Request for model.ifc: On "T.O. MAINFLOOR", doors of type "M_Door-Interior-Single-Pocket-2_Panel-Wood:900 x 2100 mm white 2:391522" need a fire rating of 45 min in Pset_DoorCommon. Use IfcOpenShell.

First a look at what the model holds.

```python
import ifcopenshell
import ifcopenshell.util.element

model = ifcopenshell.open("model.ifc")
print(model.schema)
storey = next(s for s in model.by_type("IfcBuildingStorey") if s.Name == "T.O. MAINFLOOR")
doors = [e for e in ifcopenshell.util.element.get_decomposition(storey) if e.is_a("IfcDoor")]
seen = {}
for e in doors:
    element_type = ifcopenshell.util.element.get_type(e)
    key = (element_type.Name if element_type != e and element_type else None, ifcopenshell.util.element.get_pset(e, "Pset_DoorCommon", "FireRating"))
    seen[key] = seen.get(key, 0) + 1
for (name, value), count in sorted(seen.items(), key=str):
    print(count, "x", name, "|", value)
```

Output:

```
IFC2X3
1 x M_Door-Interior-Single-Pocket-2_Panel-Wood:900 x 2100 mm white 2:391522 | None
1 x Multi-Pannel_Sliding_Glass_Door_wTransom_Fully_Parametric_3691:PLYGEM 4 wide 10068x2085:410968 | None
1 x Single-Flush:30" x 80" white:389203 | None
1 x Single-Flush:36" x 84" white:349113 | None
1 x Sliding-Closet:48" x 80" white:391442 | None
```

```python
import ifcopenshell
import ifcopenshell.api.pset
import ifcopenshell.util.element

model = ifcopenshell.open("model.ifc")

storey = next(s for s in model.by_type("IfcBuildingStorey") if s.Name == "T.O. MAINFLOOR")
doors = [e for e in ifcopenshell.util.element.get_decomposition(storey) if e.is_a("IfcDoor")]

count = 0
for e in doors:
    element_type = ifcopenshell.util.element.get_type(e)
    if element_type in (None, e) or element_type.Name != "M_Door-Interior-Single-Pocket-2_Panel-Wood:900 x 2100 mm white 2:391522":
        continue
    # add_pset returns the element's existing set when there is one.
    pset = ifcopenshell.api.pset.add_pset(model, product=e, name="Pset_DoorCommon")
    ifcopenshell.api.pset.edit_pset(model, pset=pset, properties={"FireRating": "45 min"})
    count += 1

print(count, "doors updated")

model.write("model_rev.ifc")
```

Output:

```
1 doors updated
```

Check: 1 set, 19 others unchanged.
